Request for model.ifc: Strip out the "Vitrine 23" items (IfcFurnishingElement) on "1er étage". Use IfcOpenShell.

First a look at what the model holds.

```python
import ifcopenshell
import ifcopenshell.util.element

model = ifcopenshell.open("model.ifc")
print(model.schema)
storey = next(s for s in model.by_type("IfcBuildingStorey") if s.Name == "1er étage")
furniture = [e for e in ifcopenshell.util.element.get_decomposition(storey) if e.is_a("IfcFurnishingElement")]
seen = {}
for e in furniture:
    element_type = ifcopenshell.util.element.get_type(e)
    name = element_type.Name if element_type not in (None, e) else None
    seen[name] = seen.get(name, 0) + 1
for name, count in sorted(seen.items(), key=str):
    print(count, "x", name)
```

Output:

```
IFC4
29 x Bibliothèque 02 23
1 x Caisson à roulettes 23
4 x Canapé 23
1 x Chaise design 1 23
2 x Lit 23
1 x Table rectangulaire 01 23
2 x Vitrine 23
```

```python
import ifcopenshell
import ifcopenshell.api.root
import ifcopenshell.util.element

model = ifcopenshell.open("model.ifc")

storey = next(s for s in model.by_type("IfcBuildingStorey") if s.Name == "1er étage")
furniture = [e for e in ifcopenshell.util.element.get_decomposition(storey) if e.is_a("IfcFurnishingElement")]
targets = [e for e in furniture if (t := ifcopenshell.util.element.get_type(e)) not in (None, e) and t.Name == "Vitrine 23"]

for e in targets:
    ifcopenshell.api.root.remove_product(model, product=e)
print(len(targets), "removed")

model.write("model_updated.ifc")
```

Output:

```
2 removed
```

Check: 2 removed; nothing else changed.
